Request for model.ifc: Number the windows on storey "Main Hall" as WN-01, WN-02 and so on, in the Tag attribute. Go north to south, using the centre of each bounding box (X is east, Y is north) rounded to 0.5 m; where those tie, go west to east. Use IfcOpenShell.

First a look at what the model holds.

```python
import ifcopenshell
import ifcopenshell.util.element
import ifcopenshell.util.placement

model = ifcopenshell.open("model.ifc")
print(model.schema)
storey = next(s for s in model.by_type("IfcBuildingStorey") if s.Name == "Main Hall")
windows = [e for e in ifcopenshell.util.element.get_decomposition(storey) if e.is_a("IfcWindow")]
for e in sorted(windows, key=lambda e: e.id()):
    origin = ifcopenshell.util.placement.get_local_placement(e.ObjectPlacement)[:3, 3]
    print(e.id(), e.Tag, e.Name, origin.round(2) + 0.0, sep=" | ")
```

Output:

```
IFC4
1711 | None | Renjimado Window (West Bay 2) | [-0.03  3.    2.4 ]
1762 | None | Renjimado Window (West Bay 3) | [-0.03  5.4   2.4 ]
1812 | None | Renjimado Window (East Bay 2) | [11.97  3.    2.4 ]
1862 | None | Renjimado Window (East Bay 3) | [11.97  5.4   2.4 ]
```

```python
import ifcopenshell
import ifcopenshell.geom
import ifcopenshell.util.element
import ifcopenshell.util.shape

model = ifcopenshell.open("model.ifc")
settings = ifcopenshell.geom.settings()
settings.set("use-world-coords", True)


def centre(element):
    shape = ifcopenshell.geom.create_shape(settings, element)
    return ifcopenshell.util.shape.get_bbox_centroid(shape.geometry)


storey = next(s for s in model.by_type("IfcBuildingStorey") if s.Name == "Main Hall")
windows = [e for e in ifcopenshell.util.element.get_decomposition(storey) if e.is_a("IfcWindow")]

# Insertion points can sit at a corner or the storey origin, so sort by the geometry (in metres).
centres = {e: centre(e) for e in windows}
windows.sort(key=lambda e: (-round(centres[e][1] / 0.5), centres[e][0]))

for i, e in enumerate(windows, start=1):
    number = f"WN-{i:02d}"
    e.Tag = number
    print(e.id(), number)

model.write("model_v2.ifc")
```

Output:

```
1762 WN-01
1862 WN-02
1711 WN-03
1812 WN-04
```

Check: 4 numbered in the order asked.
